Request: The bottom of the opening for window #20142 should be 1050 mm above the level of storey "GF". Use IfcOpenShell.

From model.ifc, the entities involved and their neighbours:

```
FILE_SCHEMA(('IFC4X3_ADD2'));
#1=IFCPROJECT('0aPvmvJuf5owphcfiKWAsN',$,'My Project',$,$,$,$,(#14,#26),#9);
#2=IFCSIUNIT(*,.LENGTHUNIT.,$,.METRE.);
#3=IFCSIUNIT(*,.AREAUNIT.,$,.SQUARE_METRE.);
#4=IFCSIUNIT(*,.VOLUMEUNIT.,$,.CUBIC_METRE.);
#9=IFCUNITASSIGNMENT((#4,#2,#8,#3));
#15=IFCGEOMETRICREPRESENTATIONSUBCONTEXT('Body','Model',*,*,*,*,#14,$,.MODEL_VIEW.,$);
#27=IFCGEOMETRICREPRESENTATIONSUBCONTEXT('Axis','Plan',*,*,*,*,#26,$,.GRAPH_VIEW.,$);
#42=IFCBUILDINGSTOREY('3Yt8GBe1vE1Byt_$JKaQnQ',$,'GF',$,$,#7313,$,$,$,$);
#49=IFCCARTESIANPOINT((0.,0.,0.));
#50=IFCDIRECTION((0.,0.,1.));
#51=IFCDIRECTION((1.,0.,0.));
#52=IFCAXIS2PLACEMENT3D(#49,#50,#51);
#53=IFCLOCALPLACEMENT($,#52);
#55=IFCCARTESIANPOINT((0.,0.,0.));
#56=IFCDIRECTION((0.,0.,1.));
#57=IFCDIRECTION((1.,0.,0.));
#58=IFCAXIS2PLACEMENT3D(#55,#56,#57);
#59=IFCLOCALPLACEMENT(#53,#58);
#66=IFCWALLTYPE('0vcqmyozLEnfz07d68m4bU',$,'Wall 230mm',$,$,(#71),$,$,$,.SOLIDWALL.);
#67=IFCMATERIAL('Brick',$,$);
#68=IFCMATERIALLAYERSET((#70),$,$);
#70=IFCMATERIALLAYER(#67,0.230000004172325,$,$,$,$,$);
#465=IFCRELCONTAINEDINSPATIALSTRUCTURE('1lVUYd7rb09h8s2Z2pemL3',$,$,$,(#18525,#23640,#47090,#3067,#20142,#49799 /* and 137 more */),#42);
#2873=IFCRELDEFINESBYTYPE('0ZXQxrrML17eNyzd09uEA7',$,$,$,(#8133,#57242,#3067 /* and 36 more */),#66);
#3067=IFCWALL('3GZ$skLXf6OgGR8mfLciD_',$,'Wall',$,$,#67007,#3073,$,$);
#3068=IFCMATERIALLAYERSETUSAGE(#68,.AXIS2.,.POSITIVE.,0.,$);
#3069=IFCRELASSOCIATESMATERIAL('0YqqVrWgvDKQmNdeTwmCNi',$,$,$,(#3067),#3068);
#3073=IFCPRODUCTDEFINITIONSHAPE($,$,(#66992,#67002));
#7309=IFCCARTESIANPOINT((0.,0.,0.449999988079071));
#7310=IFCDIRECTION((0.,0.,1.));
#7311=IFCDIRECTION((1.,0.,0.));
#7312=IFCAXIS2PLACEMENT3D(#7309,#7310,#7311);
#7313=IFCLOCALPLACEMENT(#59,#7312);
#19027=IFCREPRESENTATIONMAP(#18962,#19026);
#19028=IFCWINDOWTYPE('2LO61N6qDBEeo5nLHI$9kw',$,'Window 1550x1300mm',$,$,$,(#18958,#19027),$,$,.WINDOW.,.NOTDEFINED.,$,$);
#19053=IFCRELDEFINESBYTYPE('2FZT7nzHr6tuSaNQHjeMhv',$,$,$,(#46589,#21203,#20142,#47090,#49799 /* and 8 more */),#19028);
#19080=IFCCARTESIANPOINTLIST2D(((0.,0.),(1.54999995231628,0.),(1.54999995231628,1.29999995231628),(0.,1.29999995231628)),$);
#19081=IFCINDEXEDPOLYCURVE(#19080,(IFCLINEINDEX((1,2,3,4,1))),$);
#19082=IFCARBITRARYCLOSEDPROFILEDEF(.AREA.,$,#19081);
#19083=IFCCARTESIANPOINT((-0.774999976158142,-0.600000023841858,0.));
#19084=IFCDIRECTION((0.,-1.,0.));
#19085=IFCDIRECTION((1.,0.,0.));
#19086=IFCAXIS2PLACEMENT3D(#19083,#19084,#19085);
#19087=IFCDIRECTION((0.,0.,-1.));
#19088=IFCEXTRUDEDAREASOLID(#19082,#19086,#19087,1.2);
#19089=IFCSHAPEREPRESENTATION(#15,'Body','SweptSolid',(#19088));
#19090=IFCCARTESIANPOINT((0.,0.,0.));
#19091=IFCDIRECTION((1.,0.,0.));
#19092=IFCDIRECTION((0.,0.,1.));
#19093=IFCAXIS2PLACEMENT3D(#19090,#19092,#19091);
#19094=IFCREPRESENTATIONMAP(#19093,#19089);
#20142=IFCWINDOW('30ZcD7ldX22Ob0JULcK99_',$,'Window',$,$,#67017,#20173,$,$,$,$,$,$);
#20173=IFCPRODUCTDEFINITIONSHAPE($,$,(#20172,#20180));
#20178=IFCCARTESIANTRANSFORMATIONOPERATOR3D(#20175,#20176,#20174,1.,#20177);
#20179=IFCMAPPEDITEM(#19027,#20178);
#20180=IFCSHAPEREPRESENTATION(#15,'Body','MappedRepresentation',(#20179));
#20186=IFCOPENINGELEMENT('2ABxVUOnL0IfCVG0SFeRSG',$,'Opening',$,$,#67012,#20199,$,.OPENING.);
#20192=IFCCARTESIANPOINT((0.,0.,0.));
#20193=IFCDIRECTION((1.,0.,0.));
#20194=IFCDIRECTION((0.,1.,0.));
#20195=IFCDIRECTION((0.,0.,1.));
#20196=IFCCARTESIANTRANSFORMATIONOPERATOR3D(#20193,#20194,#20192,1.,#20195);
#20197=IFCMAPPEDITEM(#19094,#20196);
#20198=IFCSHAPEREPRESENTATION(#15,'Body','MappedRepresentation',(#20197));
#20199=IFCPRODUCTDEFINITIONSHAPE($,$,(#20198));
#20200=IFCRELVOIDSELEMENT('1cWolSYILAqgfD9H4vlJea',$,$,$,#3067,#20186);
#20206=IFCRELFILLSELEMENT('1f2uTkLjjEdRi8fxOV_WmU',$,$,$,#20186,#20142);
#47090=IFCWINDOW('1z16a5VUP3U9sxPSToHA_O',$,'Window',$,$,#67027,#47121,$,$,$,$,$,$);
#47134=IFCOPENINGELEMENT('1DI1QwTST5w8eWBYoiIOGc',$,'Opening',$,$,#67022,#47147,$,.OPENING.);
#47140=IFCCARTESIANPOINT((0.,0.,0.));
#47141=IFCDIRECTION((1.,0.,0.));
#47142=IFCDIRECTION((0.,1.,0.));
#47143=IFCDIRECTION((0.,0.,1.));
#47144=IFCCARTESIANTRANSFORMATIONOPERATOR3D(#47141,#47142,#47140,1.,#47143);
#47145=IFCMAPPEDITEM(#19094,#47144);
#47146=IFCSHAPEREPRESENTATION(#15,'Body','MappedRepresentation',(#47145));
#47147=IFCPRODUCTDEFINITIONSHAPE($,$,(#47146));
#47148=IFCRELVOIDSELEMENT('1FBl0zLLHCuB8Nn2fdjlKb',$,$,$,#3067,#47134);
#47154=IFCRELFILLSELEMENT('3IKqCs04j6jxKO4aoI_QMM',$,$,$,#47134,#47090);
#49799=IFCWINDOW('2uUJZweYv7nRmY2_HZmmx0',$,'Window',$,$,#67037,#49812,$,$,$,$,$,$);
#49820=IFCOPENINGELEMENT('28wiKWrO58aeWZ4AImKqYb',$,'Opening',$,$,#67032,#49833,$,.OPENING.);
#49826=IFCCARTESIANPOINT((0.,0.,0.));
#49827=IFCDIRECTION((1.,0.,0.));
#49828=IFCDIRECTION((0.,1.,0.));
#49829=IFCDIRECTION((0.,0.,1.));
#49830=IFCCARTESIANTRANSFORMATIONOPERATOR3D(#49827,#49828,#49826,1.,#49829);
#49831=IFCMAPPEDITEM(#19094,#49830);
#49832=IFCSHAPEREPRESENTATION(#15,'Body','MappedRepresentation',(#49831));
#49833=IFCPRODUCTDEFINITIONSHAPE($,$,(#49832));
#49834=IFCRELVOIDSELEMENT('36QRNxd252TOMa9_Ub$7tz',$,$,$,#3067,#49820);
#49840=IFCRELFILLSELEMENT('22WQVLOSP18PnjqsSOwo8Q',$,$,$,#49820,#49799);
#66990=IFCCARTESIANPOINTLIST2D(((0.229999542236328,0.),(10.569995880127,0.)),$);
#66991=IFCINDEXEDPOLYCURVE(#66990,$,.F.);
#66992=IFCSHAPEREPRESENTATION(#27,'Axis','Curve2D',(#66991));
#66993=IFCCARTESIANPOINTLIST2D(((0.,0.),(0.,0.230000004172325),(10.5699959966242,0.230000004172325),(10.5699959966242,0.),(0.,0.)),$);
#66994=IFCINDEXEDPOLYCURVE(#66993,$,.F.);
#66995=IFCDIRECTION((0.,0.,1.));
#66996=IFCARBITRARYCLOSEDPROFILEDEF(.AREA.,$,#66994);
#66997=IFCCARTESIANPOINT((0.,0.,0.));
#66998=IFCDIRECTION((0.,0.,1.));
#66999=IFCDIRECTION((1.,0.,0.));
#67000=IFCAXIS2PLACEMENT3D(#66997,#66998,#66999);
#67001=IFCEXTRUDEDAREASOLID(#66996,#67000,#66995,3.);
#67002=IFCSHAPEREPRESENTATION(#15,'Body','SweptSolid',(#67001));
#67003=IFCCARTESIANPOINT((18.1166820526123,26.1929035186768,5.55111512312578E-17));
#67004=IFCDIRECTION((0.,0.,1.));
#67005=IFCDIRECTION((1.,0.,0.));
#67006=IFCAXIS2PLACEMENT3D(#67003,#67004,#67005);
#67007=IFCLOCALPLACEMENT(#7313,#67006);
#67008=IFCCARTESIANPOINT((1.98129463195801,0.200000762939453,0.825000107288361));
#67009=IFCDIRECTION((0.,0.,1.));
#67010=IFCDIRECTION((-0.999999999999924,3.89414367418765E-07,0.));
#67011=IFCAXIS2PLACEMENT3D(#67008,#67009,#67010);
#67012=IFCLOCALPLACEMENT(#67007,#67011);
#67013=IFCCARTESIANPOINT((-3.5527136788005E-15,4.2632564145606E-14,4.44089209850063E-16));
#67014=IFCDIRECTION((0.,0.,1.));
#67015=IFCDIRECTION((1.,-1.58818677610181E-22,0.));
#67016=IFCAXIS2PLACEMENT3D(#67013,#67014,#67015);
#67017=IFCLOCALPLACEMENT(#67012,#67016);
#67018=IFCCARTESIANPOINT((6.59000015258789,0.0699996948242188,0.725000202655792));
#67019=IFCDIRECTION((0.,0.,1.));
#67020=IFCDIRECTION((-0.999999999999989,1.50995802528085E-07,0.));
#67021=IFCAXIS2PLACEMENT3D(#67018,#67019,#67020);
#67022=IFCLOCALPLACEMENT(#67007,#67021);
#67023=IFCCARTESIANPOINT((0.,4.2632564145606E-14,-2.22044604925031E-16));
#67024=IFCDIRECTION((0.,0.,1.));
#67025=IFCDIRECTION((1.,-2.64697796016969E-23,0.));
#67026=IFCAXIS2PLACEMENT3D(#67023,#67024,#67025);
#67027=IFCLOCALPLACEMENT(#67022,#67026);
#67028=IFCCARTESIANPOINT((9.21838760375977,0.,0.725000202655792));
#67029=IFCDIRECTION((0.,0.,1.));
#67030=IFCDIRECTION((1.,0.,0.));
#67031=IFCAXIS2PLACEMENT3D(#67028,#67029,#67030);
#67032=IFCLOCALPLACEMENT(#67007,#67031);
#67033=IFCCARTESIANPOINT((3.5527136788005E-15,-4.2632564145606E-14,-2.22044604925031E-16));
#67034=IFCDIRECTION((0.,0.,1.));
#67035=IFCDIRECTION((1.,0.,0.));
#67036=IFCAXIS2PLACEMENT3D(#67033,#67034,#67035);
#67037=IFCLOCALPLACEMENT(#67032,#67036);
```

```python
import numpy as np
import ifcopenshell
import ifcopenshell.api.geometry
import ifcopenshell.geom
import ifcopenshell.util.element
import ifcopenshell.util.placement
import ifcopenshell.util.shape
import ifcopenshell.util.unit

model = ifcopenshell.open("model.ifc")
unit_scale = ifcopenshell.util.unit.calculate_unit_scale(model)

window = model.by_guid("30ZcD7ldX22Ob0JULcK99_")
opening = window.FillsVoids[0].RelatingOpeningElement
storey = ifcopenshell.util.element.get_container(window, ifc_class="IfcBuildingStorey")
level = ifcopenshell.util.placement.get_local_placement(storey.ObjectPlacement)[2, 3]

# The opening's origin need not be at the sill, so measure its lowest point.
shape = ifcopenshell.geom.create_shape(ifcopenshell.geom.settings(), opening)
bottom = ifcopenshell.util.shape.get_shape_bottom_elevation(shape, shape.geometry) / unit_scale
dz = level + 1.05 / unit_scale - bottom

shift = np.array([0.0, 0.0, dz])
# The window is placed relative to its opening, so it follows when the opening moves.
matrix = ifcopenshell.util.placement.get_local_placement(opening.ObjectPlacement)
matrix[:3, 3] += shift
ifcopenshell.api.geometry.edit_object_placement(
    model, product=opening, matrix=matrix, is_si=False, should_transform_children=True
)

print(f"moved by {dz * unit_scale:+.3f} m")

model.write("model-out.ifc")
```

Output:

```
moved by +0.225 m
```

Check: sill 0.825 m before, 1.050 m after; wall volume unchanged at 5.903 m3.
